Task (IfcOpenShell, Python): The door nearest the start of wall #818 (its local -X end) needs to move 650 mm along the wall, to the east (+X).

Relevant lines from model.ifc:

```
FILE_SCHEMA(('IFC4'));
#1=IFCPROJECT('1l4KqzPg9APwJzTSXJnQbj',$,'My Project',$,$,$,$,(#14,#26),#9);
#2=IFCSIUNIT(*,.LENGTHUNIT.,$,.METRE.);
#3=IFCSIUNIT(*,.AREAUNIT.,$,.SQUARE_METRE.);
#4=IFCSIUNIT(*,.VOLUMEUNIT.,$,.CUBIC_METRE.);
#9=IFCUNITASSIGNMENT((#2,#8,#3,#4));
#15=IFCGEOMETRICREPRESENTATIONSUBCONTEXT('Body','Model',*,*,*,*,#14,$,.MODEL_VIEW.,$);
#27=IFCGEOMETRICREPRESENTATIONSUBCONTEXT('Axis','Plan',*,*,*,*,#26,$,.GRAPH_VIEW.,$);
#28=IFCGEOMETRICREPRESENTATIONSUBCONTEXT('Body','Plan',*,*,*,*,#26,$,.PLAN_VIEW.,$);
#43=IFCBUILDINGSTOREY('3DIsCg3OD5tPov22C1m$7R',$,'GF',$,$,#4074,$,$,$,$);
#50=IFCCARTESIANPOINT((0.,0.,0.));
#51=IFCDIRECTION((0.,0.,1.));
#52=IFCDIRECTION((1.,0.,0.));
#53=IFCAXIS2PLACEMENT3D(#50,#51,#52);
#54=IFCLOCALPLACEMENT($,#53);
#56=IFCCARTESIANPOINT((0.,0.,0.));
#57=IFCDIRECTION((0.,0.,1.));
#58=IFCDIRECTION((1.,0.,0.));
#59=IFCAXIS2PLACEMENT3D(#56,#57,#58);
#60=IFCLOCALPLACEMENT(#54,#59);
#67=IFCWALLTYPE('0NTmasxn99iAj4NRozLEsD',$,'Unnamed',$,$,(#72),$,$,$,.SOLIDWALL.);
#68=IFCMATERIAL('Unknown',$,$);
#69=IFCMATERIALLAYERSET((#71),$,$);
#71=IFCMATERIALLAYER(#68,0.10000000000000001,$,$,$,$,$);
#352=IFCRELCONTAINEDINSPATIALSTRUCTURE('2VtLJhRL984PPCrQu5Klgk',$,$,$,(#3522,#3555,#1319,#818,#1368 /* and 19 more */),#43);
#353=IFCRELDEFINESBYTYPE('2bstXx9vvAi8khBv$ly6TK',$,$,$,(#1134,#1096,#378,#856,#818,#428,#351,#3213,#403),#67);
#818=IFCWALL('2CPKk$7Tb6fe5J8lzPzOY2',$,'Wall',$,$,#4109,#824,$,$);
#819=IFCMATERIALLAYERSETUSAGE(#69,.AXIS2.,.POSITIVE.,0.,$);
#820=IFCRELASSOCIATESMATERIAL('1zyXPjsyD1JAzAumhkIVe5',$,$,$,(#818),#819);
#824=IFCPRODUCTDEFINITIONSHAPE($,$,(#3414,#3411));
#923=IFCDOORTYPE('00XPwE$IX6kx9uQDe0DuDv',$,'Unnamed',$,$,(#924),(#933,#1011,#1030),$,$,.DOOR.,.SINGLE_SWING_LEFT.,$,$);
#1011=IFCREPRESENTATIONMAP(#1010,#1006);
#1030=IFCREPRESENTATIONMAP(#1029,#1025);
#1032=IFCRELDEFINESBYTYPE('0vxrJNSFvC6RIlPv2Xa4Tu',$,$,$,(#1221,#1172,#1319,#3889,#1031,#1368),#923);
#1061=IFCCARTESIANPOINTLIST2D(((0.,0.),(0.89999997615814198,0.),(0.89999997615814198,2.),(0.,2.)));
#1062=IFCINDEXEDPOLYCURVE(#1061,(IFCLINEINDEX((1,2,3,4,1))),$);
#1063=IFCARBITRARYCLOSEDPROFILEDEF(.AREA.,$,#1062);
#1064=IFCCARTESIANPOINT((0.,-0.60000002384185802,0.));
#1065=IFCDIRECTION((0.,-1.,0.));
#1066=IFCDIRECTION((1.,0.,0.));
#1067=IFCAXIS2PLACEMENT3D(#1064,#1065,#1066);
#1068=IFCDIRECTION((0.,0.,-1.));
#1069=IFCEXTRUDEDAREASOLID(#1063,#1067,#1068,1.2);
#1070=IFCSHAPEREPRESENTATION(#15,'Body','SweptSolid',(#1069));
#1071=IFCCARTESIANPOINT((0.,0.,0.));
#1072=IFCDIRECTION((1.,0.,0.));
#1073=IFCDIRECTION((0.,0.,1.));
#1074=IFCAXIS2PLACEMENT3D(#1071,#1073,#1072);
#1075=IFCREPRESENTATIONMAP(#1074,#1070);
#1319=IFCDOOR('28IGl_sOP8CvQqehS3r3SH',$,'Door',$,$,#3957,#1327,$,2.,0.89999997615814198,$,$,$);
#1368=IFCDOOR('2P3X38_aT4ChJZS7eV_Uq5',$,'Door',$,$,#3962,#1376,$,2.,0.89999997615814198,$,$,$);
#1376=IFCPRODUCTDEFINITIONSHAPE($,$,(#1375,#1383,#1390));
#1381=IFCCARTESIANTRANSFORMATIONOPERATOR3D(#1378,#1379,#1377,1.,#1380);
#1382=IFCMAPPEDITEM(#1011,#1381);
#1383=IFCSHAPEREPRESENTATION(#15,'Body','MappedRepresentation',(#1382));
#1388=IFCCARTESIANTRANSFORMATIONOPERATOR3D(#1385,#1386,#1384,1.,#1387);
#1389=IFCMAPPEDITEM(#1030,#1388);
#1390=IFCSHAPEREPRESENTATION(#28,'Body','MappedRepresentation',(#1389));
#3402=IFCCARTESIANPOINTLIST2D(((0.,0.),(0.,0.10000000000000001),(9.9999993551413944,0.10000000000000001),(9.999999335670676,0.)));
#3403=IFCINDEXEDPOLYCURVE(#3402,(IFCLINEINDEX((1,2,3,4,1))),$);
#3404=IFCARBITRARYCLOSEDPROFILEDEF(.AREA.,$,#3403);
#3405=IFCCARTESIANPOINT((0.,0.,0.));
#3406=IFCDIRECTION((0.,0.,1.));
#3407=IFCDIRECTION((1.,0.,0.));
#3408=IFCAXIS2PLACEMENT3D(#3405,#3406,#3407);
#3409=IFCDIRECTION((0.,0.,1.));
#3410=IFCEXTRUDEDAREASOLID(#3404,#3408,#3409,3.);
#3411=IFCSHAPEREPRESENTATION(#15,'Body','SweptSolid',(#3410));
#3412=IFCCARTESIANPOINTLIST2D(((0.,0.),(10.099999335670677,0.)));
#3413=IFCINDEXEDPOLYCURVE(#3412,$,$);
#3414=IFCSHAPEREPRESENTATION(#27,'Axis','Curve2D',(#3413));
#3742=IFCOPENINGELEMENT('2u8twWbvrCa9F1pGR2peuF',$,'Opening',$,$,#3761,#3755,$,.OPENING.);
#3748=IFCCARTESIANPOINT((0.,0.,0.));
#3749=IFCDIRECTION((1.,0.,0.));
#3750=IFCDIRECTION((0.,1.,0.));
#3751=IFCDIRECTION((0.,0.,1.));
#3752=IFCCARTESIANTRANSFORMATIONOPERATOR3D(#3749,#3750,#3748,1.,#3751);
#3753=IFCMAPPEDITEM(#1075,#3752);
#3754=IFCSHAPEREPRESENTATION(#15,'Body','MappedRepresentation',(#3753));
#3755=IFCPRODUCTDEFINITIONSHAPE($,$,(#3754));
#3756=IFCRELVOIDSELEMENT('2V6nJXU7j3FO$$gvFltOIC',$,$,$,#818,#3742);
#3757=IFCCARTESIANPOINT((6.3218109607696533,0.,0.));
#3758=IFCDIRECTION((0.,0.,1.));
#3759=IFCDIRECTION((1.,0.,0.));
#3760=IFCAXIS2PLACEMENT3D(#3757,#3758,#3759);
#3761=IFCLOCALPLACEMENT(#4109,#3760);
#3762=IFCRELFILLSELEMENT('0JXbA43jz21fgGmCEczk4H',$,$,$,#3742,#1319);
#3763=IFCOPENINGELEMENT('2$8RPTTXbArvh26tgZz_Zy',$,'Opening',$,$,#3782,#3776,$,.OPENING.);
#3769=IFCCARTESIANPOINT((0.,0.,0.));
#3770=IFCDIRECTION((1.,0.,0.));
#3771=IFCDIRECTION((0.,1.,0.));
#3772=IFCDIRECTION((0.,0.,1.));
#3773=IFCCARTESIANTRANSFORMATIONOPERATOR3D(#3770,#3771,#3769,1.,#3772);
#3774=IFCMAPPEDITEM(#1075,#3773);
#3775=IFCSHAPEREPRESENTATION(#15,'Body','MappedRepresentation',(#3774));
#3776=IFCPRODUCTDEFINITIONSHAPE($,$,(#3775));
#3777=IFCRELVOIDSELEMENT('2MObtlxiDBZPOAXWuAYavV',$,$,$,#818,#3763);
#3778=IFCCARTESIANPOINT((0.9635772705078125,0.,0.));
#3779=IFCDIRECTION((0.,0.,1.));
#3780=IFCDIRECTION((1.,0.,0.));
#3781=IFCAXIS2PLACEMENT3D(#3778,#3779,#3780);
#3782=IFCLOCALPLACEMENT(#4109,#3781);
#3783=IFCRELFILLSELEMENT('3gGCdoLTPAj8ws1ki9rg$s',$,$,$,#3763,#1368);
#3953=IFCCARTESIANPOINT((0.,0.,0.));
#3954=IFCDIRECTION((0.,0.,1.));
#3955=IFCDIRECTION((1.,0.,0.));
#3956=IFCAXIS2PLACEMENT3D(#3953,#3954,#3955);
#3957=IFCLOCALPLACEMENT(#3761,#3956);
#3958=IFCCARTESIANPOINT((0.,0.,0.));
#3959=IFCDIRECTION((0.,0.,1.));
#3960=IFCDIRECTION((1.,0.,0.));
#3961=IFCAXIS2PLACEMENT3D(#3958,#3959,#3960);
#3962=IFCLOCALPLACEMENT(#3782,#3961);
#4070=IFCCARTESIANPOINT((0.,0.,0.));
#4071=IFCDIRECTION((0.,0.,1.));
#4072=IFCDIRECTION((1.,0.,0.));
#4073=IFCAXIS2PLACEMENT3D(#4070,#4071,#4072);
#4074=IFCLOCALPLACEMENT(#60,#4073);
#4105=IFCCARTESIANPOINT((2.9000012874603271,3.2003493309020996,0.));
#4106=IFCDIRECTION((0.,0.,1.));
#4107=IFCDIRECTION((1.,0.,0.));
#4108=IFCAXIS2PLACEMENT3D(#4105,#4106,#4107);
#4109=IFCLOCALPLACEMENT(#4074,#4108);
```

```python
import ifcopenshell
import ifcopenshell.api.geometry
import ifcopenshell.util.placement

model = ifcopenshell.open("model.ifc")

door = model.by_id(1368)
opening = door.FillsVoids[0].RelatingOpeningElement
wall = opening.VoidsElements[0].RelatingBuildingElement

wall_matrix = ifcopenshell.util.placement.get_local_placement(wall.ObjectPlacement)
shift = wall_matrix[:3, 0] * 0.65
before = ifcopenshell.util.placement.get_local_placement(door.ObjectPlacement)[:3, 3].copy()

# The door is placed relative to its opening, so it follows when the opening moves.
matrix = ifcopenshell.util.placement.get_local_placement(opening.ObjectPlacement)
matrix[:3, 3] += shift
ifcopenshell.api.geometry.edit_object_placement(
    model, product=opening, matrix=matrix, is_si=False, should_transform_children=True
)

after = ifcopenshell.util.placement.get_local_placement(door.ObjectPlacement)[:3, 3]
print("door moved by", (after - before).round(3) + 0.0)

model.write("model_v2.ifc")
```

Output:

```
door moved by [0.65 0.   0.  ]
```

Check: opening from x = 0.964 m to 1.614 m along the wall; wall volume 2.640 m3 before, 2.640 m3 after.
